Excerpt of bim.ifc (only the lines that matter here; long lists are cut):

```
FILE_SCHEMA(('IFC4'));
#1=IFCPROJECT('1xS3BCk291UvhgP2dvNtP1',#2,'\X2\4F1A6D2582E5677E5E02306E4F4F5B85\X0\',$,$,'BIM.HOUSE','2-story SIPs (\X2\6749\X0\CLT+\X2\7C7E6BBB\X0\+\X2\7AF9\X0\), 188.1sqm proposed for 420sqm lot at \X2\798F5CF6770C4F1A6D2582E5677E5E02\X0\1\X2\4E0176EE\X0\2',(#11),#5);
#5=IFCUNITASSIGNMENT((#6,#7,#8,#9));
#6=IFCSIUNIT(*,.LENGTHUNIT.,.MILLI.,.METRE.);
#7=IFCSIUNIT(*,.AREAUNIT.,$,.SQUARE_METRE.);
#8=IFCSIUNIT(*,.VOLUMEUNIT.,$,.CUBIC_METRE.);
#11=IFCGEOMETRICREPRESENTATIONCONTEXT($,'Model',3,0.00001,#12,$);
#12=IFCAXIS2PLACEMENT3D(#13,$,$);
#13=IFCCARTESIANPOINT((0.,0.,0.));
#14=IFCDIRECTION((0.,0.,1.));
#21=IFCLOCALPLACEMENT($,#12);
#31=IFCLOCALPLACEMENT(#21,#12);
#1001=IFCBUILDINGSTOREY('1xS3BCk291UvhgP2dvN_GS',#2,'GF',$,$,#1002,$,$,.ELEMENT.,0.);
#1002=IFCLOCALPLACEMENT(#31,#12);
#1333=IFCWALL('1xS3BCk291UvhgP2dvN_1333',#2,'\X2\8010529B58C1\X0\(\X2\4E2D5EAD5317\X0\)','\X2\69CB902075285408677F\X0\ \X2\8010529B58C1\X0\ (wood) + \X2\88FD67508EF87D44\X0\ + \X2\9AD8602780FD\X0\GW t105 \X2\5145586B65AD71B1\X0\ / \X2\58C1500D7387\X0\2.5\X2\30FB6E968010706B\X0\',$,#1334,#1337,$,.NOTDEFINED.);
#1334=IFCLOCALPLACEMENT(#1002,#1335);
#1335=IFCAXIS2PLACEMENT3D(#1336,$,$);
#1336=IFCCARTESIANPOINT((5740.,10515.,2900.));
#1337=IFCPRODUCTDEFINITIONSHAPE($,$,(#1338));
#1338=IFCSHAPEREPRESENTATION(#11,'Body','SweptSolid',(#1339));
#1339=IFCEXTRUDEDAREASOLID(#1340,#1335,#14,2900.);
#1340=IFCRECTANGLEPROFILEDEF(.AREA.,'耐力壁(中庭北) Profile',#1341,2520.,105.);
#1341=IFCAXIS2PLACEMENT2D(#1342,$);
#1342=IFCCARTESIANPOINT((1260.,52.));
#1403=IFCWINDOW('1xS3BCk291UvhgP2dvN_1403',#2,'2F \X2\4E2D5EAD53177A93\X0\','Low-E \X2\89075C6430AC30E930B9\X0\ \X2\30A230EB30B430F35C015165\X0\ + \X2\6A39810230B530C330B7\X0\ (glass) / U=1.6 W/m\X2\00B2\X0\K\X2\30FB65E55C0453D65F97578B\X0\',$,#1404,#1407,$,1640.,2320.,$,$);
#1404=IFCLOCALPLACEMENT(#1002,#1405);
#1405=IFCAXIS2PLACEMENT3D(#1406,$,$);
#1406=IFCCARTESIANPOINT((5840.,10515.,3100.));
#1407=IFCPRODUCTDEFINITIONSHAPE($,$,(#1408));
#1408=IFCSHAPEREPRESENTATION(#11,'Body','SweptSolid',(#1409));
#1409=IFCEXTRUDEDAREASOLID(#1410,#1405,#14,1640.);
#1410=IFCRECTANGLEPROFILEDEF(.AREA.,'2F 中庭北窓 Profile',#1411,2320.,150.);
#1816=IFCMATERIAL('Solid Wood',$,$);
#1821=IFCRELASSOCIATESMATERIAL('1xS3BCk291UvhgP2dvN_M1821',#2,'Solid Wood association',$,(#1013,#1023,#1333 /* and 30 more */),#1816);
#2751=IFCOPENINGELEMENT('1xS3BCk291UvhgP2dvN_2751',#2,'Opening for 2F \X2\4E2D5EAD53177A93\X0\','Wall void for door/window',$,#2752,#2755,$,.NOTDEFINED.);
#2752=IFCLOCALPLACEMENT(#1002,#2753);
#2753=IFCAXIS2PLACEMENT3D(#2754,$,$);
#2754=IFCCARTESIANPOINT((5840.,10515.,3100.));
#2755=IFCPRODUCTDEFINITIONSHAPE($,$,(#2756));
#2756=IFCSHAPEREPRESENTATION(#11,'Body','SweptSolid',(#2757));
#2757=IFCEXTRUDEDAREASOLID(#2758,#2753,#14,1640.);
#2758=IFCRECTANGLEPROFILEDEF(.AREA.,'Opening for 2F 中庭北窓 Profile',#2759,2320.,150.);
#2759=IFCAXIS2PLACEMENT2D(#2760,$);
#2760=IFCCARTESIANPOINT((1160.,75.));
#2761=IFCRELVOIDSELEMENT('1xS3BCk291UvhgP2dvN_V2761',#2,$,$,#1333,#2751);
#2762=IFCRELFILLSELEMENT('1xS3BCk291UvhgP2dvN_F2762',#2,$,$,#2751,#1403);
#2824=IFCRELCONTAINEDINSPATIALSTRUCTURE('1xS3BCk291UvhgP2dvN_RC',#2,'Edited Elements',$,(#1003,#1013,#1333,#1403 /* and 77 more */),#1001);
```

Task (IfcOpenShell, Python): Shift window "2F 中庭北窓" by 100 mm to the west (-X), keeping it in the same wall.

```python
import ifcopenshell
import ifcopenshell.api.geometry
import ifcopenshell.util.placement

model = ifcopenshell.open("bim.ifc")

window = model.by_guid("1xS3BCk291UvhgP2dvN_1403")
opening = window.FillsVoids[0].RelatingOpeningElement
wall = opening.VoidsElements[0].RelatingBuildingElement

wall_matrix = ifcopenshell.util.placement.get_local_placement(wall.ObjectPlacement)
shift = wall_matrix[:3, 0] * -100.0
before = ifcopenshell.util.placement.get_local_placement(window.ObjectPlacement)[:3, 3].copy()

# The window is not placed relative to its opening, so move both.
for product in (opening, window):
    matrix = ifcopenshell.util.placement.get_local_placement(product.ObjectPlacement)
    matrix[:3, 3] += shift
    ifcopenshell.api.geometry.edit_object_placement(model, product=product, matrix=matrix, is_si=False)

after = ifcopenshell.util.placement.get_local_placement(window.ObjectPlacement)[:3, 3]
print("window moved by", (after - before).round(3) + 0.0)

model.write("bim_rev.ifc")
```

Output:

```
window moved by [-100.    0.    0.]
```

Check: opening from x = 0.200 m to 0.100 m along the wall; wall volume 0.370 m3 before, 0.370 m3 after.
